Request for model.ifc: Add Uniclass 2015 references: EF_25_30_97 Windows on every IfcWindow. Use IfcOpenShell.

First a look at what the model holds.

```python
import ifcopenshell

model = ifcopenshell.open("model.ifc")
print(model.schema)
print("classifications:", [c.Name for c in model.by_type("IfcClassification")])
for ifc_class in ("IfcDoor", "IfcRoof", "IfcStair", "IfcWall", "IfcWindow"):
    print(ifc_class, len(model.by_type(ifc_class)))
```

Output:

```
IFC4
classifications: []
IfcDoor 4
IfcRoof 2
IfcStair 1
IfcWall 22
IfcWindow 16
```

```python
import ifcopenshell
import ifcopenshell.api.classification

model = ifcopenshell.open("model.ifc")

system = ifcopenshell.api.classification.add_classification(model, classification="Uniclass 2015")

codes = {
    "IfcWindow": ("EF_25_30_97", "Windows"),
}
for ifc_class, (code, name) in codes.items():
    products = model.by_type(ifc_class)
    ifcopenshell.api.classification.add_reference(
        model, products=products, classification=system, identification=code, name=name
    )
    print(code, len(products))

model.write("model_rev.ifc")
```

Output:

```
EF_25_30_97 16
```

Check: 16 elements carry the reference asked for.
